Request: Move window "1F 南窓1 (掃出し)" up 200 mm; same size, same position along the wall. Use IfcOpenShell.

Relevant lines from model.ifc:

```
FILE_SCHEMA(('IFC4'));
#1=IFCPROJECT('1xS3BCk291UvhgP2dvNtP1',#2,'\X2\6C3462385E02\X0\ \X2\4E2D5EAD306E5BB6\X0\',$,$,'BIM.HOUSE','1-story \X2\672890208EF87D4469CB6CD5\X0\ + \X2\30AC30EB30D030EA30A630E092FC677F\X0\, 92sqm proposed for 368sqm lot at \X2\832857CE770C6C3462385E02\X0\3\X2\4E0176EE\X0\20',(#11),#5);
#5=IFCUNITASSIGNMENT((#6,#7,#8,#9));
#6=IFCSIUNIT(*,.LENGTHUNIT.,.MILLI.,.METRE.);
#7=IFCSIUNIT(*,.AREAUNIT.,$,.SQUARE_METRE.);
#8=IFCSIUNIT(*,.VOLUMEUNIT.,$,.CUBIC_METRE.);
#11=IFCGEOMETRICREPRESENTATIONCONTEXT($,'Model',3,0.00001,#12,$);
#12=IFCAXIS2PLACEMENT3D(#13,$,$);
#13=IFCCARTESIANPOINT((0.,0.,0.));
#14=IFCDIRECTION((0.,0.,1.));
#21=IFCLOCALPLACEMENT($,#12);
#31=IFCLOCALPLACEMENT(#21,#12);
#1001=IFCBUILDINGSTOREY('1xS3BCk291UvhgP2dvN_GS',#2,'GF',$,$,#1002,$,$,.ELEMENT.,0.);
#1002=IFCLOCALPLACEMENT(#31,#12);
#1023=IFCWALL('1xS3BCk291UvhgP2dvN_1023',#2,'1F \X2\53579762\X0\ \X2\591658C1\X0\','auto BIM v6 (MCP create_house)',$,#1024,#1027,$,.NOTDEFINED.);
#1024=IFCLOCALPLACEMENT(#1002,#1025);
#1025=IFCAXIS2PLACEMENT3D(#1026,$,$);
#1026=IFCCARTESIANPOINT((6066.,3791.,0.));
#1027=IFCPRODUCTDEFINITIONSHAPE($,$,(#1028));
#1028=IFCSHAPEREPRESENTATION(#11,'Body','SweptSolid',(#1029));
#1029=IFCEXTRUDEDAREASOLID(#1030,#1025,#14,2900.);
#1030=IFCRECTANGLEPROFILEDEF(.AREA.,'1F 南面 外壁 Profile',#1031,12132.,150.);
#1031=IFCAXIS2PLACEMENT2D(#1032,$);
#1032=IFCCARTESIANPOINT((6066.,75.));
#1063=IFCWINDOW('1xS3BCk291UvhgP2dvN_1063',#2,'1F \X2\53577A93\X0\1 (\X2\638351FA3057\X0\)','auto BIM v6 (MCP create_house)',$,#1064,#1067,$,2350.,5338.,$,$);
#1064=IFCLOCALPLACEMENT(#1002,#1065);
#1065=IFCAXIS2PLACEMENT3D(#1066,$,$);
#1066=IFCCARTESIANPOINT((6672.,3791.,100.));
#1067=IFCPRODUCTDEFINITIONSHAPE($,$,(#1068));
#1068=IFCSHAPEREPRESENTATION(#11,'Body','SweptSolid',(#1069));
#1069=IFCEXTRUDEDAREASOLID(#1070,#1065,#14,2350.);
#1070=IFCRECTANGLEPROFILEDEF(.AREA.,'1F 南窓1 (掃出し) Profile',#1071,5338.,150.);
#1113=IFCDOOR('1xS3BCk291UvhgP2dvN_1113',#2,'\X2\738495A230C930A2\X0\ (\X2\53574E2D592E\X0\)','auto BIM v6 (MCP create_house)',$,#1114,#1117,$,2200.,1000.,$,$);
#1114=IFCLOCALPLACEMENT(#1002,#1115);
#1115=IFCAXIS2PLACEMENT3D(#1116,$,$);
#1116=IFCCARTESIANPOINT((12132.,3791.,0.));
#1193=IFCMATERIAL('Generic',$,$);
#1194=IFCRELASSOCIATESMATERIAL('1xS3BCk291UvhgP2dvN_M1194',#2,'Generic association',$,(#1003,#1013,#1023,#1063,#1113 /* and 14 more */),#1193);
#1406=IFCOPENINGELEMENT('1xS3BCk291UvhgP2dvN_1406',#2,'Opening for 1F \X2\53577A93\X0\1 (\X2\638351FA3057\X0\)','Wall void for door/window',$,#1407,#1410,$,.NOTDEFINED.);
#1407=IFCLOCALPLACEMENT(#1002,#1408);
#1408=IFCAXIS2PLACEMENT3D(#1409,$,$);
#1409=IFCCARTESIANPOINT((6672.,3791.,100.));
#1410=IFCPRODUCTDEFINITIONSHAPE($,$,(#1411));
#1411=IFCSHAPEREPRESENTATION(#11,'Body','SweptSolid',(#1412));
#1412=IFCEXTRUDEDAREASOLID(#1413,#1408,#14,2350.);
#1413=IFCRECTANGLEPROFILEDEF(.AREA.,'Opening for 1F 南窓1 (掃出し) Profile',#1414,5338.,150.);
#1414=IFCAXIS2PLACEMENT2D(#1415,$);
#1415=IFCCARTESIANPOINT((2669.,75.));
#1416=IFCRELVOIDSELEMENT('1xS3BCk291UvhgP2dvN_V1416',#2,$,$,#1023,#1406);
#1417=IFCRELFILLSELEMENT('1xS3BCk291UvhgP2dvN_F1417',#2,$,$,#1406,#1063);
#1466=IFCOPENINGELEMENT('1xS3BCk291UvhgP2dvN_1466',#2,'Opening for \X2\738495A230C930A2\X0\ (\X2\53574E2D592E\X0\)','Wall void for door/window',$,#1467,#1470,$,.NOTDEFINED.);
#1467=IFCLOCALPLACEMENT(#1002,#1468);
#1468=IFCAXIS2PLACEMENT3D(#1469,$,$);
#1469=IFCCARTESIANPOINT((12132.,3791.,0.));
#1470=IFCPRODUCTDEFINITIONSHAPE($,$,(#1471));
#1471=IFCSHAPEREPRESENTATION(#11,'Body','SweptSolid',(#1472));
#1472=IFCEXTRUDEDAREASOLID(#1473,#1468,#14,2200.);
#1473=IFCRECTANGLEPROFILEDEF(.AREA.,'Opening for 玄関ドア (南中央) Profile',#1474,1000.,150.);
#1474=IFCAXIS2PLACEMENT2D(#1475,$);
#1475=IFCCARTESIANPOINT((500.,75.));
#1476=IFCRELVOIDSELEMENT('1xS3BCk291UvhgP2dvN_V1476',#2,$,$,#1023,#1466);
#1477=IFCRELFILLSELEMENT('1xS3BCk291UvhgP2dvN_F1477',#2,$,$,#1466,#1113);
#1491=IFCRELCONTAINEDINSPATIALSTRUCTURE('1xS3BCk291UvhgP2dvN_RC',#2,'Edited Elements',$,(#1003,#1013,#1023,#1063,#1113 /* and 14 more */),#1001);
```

```python
import numpy as np
import ifcopenshell
import ifcopenshell.api.geometry
import ifcopenshell.util.placement
import ifcopenshell.util.unit

model = ifcopenshell.open("model.ifc")
unit_scale = ifcopenshell.util.unit.calculate_unit_scale(model)

window = model.by_id(1063)
opening = window.FillsVoids[0].RelatingOpeningElement
dz = 200.0

shift = np.array([0.0, 0.0, dz])
# The window is not placed relative to its opening, so move both.
for product in (opening, window):
    matrix = ifcopenshell.util.placement.get_local_placement(product.ObjectPlacement)
    matrix[:3, 3] += shift
    ifcopenshell.api.geometry.edit_object_placement(model, product=product, matrix=matrix, is_si=False)

print(f"moved by {dz * unit_scale:+.3f} m")

model.write("model_updated.ifc")
```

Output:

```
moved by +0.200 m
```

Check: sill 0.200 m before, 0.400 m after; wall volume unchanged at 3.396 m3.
